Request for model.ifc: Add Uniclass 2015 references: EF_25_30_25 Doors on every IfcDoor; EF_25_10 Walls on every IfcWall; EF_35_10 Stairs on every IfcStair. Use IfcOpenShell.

First a look at what the model holds.

```python
import ifcopenshell

model = ifcopenshell.open("model.ifc")
print(model.schema)
print("classifications:", [c.Name for c in model.by_type("IfcClassification")])
for ifc_class in ("IfcDoor", "IfcRoof", "IfcStair", "IfcWall", "IfcWindow"):
    print(ifc_class, len(model.by_type(ifc_class)))
```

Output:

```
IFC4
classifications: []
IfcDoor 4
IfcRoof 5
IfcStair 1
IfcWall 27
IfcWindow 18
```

```python
import ifcopenshell
import ifcopenshell.api.classification

model = ifcopenshell.open("model.ifc")

system = ifcopenshell.api.classification.add_classification(model, classification="Uniclass 2015")

codes = {
    "IfcDoor": ("EF_25_30_25", "Doors"),
    "IfcWall": ("EF_25_10", "Walls"),
    "IfcStair": ("EF_35_10", "Stairs"),
}
for ifc_class, (code, name) in codes.items():
    products = model.by_type(ifc_class)
    ifcopenshell.api.classification.add_reference(
        model, products=products, classification=system, identification=code, name=name
    )
    print(code, len(products))

model.write("model_updated.ifc")
```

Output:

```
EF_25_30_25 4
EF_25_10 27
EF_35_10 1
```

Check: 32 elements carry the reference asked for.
